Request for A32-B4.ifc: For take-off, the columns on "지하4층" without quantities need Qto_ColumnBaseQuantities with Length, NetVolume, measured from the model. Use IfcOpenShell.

First a look at what the model holds.

```python
import ifcopenshell
import ifcopenshell.util.element
import ifcopenshell.util.unit

model = ifcopenshell.open("A32-B4.ifc")
print(model.schema)
for unit_type in ("LENGTHUNIT", "AREAUNIT", "VOLUMEUNIT"):
    print(unit_type, ifcopenshell.util.unit.calculate_unit_scale(model, unit_type))
storey = next(s for s in model.by_type("IfcBuildingStorey") if s.Name == "지하4층")
columns = [e for e in ifcopenshell.util.element.get_decomposition(storey) if e.is_a("IfcColumn")]
for e in sorted(columns, key=lambda e: e.id()):
    print(e.id(), e.is_a(), e.Name, list(ifcopenshell.util.element.get_psets(e, qtos_only=True)), sep=" | ")
```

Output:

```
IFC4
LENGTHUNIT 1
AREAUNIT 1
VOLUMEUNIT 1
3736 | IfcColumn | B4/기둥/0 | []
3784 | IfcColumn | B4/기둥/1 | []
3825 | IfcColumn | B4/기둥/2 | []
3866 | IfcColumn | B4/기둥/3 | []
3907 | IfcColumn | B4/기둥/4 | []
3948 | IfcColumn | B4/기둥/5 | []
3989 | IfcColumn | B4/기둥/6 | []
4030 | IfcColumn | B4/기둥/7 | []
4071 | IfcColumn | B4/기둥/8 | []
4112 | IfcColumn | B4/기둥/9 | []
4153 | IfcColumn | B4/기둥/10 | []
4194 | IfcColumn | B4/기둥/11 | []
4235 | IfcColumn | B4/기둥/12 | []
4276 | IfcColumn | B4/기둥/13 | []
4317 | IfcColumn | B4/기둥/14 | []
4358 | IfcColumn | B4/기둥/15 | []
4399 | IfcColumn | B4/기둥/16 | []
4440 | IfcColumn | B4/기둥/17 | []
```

```python
import ifcopenshell
import ifcopenshell.api.pset
import ifcopenshell.geom
import ifcopenshell.util.element
import ifcopenshell.util.shape
import ifcopenshell.util.unit

model = ifcopenshell.open("A32-B4.ifc")
unit_scale = ifcopenshell.util.unit.calculate_unit_scale(model)
volume_scale = ifcopenshell.util.unit.calculate_unit_scale(model, "VOLUMEUNIT")
settings = ifcopenshell.geom.settings()

storey = next(s for s in model.by_type("IfcBuildingStorey") if s.Name == "지하4층")
columns = [e for e in ifcopenshell.util.element.get_decomposition(storey) if e.is_a("IfcColumn")]

for e in sorted(columns, key=lambda e: e.id()):
    if ifcopenshell.util.element.get_psets(e, qtos_only=True, should_inherit=False):
        continue
    # Geometry comes back in metres, in the element's own axes.
    shape = ifcopenshell.geom.create_shape(settings, e)
    values = {
        "Length": ifcopenshell.util.shape.get_z(shape.geometry) / unit_scale,
        "NetVolume": ifcopenshell.util.shape.get_volume(shape.geometry) / volume_scale,
    }
    qto = ifcopenshell.api.pset.add_qto(model, product=e, name="Qto_ColumnBaseQuantities")
    ifcopenshell.api.pset.edit_qto(model, qto=qto, properties=values)
    print(e.id(), {k: round(v, 3) for k, v in values.items()})

model.write("A32-B4_v2.ifc")
```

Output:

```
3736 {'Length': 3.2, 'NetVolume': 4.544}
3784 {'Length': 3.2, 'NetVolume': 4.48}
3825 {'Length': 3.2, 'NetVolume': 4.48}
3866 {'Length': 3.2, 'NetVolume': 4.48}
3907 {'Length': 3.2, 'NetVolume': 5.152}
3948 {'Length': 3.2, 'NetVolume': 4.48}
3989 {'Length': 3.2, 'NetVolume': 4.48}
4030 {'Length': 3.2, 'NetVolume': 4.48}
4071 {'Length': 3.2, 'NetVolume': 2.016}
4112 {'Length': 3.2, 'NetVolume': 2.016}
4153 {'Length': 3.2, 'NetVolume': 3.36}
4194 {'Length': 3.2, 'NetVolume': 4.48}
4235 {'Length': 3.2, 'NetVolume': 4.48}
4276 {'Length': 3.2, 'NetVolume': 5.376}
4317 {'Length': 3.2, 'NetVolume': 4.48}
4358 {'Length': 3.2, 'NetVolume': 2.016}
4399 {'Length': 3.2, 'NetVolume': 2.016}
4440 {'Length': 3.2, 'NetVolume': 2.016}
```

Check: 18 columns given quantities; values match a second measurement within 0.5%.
